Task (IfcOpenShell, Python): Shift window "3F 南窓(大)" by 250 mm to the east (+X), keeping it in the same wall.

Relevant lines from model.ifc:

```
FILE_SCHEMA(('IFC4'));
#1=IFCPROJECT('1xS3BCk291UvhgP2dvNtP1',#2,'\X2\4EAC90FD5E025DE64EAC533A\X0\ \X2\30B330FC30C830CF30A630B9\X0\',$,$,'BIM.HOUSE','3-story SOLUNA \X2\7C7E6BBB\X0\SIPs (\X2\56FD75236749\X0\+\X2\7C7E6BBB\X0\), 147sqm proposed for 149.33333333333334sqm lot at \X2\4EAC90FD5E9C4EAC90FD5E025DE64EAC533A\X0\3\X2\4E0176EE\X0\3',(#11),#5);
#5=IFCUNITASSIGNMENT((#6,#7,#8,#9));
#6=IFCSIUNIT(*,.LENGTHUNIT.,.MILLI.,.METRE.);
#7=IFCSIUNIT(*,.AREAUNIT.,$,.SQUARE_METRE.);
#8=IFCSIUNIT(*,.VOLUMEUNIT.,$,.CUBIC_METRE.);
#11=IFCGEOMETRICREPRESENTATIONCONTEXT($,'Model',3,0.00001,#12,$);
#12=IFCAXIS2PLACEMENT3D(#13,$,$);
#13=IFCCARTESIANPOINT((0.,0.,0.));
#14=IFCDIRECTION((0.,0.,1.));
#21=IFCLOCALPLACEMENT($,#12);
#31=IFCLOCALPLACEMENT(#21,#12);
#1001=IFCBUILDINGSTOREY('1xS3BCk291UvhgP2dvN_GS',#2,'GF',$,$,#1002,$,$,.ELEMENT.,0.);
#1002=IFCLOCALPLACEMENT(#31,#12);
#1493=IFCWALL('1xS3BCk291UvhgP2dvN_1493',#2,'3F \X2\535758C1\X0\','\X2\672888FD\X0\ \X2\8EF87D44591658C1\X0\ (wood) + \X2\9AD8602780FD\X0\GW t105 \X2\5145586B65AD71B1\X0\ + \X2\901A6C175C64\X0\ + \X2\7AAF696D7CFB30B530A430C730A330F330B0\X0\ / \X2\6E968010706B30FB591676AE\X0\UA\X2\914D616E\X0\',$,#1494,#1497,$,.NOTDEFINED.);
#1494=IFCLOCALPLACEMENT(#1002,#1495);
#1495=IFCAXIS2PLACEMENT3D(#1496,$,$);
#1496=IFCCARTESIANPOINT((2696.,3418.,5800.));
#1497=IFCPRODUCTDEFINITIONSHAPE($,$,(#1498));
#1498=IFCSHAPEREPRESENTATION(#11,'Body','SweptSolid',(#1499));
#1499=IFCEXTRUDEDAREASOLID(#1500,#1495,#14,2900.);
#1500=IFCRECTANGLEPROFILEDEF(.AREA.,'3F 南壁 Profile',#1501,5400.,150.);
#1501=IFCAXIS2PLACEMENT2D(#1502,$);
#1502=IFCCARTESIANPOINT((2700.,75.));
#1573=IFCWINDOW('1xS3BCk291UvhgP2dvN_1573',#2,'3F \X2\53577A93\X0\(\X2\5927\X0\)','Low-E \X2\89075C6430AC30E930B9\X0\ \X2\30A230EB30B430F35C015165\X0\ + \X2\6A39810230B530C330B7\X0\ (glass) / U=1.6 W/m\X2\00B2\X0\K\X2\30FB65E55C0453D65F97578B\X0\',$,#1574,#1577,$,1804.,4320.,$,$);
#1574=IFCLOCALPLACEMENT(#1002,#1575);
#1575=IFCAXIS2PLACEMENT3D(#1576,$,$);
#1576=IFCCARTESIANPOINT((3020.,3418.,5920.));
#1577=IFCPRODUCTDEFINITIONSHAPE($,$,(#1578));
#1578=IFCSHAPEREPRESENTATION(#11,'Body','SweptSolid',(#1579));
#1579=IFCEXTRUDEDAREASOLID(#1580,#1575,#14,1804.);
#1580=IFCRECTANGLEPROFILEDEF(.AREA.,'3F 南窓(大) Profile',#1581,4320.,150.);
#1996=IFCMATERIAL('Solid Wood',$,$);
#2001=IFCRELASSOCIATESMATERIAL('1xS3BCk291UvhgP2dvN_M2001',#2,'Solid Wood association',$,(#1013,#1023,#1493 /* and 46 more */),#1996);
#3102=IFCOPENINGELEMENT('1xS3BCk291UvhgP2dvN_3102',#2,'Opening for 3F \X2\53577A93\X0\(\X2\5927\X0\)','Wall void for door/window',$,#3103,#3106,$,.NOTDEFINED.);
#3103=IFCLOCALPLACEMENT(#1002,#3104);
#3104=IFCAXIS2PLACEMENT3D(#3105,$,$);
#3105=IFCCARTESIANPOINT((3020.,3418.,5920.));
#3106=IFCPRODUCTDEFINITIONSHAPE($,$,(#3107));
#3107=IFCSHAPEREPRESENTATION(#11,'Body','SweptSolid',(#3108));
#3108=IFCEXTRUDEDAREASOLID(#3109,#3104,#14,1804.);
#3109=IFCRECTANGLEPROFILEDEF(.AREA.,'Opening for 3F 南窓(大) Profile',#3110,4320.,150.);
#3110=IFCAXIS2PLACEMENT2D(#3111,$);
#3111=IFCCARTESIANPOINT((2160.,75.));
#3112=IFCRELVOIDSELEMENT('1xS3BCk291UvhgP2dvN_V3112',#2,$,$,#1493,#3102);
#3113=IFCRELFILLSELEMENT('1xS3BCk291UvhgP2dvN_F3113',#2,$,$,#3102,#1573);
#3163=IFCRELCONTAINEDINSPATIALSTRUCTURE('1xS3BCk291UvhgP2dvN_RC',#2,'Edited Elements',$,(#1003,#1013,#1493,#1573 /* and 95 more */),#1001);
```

```python
import ifcopenshell
import ifcopenshell.api.geometry
import ifcopenshell.util.placement
import ifcopenshell.util.unit

model = ifcopenshell.open("model.ifc")
unit_scale = ifcopenshell.util.unit.calculate_unit_scale(model)

window = model.by_id(1573)
opening = window.FillsVoids[0].RelatingOpeningElement
wall = opening.VoidsElements[0].RelatingBuildingElement

wall_matrix = ifcopenshell.util.placement.get_local_placement(wall.ObjectPlacement)
shift = wall_matrix[:3, 0] * 0.25 / unit_scale
before = ifcopenshell.util.placement.get_local_placement(window.ObjectPlacement)[:3, 3].copy()

# The window is not placed relative to its opening, so move both.
for product in (opening, window):
    matrix = ifcopenshell.util.placement.get_local_placement(product.ObjectPlacement)
    matrix[:3, 3] += shift
    ifcopenshell.api.geometry.edit_object_placement(model, product=product, matrix=matrix, is_si=False)

after = ifcopenshell.util.placement.get_local_placement(window.ObjectPlacement)[:3, 3]
print("window moved by", (after - before).round(3) + 0.0)

model.write("model_v2.ifc")
```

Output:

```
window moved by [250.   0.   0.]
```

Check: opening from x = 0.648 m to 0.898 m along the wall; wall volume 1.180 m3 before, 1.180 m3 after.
